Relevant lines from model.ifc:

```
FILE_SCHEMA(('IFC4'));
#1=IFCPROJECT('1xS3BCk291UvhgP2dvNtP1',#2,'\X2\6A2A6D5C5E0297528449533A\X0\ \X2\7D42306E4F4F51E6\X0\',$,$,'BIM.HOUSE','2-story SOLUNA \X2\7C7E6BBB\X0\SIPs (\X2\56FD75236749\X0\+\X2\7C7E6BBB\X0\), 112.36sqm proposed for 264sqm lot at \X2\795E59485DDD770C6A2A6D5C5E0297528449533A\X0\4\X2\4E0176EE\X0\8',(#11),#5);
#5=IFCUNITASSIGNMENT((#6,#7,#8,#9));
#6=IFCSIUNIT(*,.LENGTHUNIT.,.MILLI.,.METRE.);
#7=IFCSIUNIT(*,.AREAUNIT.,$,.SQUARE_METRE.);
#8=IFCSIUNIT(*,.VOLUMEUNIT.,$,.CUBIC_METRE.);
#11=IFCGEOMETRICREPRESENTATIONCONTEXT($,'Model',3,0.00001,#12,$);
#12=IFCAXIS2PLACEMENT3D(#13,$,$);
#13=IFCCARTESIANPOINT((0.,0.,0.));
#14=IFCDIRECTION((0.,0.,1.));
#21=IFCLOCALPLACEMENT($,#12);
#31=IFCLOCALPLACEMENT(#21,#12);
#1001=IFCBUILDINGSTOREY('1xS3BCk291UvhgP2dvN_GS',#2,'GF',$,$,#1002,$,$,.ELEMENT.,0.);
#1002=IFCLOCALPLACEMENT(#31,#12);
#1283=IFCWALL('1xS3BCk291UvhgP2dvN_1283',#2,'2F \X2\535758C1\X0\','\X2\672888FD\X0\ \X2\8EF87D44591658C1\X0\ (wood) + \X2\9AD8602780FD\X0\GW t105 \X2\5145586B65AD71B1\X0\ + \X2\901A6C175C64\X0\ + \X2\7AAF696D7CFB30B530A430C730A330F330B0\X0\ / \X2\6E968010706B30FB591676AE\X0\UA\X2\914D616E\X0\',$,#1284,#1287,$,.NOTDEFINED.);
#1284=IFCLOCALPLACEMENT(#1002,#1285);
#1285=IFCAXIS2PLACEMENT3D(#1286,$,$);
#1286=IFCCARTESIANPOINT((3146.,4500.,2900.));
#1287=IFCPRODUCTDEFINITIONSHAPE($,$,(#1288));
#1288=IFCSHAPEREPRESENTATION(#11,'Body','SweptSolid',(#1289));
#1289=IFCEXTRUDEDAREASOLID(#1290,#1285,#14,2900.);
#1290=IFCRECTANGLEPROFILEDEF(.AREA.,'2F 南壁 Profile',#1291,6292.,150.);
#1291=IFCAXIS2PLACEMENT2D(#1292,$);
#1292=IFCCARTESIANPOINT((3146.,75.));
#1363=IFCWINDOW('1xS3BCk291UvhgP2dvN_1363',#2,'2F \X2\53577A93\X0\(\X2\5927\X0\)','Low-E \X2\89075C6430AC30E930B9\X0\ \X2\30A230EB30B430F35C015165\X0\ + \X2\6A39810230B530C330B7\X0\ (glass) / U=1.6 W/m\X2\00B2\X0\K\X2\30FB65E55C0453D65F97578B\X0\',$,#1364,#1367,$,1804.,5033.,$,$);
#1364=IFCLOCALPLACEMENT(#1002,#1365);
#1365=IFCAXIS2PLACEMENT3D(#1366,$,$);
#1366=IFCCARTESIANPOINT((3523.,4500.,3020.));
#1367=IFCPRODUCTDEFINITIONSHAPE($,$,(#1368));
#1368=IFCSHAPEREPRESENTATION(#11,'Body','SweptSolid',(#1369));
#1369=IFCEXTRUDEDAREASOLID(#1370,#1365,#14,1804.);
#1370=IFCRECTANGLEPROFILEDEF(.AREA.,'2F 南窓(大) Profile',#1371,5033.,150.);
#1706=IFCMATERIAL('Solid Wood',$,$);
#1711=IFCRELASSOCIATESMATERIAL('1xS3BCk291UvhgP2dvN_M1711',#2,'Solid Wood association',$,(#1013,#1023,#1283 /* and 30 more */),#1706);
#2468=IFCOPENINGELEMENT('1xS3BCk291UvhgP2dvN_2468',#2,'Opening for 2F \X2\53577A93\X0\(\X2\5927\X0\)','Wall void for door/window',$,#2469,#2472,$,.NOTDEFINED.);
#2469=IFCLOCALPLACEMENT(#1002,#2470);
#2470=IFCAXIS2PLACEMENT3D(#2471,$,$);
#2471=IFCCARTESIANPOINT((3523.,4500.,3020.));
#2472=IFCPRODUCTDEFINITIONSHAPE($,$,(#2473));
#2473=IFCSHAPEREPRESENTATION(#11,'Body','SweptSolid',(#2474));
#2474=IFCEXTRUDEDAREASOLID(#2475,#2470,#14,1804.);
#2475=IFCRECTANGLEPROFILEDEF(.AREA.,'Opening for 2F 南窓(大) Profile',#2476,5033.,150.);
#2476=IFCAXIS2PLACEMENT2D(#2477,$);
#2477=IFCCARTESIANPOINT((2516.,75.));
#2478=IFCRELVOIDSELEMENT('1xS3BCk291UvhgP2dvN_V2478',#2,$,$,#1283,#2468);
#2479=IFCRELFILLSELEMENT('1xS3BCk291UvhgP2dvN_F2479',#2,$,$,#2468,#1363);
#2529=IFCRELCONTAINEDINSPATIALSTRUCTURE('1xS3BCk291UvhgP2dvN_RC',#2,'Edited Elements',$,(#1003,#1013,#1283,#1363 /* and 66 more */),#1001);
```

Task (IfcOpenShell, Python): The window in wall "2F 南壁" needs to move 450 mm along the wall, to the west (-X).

```python
import ifcopenshell
import ifcopenshell.api.geometry
import ifcopenshell.util.placement

model = ifcopenshell.open("model.ifc")

window = model.by_guid("1xS3BCk291UvhgP2dvN_1363")
opening = window.FillsVoids[0].RelatingOpeningElement
wall = opening.VoidsElements[0].RelatingBuildingElement

wall_matrix = ifcopenshell.util.placement.get_local_placement(wall.ObjectPlacement)
shift = wall_matrix[:3, 0] * -450.0
before = ifcopenshell.util.placement.get_local_placement(window.ObjectPlacement)[:3, 3].copy()

# The window is not placed relative to its opening, so move both.
for product in (opening, window):
    matrix = ifcopenshell.util.placement.get_local_placement(product.ObjectPlacement)
    matrix[:3, 3] += shift
    ifcopenshell.api.geometry.edit_object_placement(model, product=product, matrix=matrix, is_si=False)

after = ifcopenshell.util.placement.get_local_placement(window.ObjectPlacement)[:3, 3]
print("window moved by", (after - before).round(3) + 0.0)

model.write("model_updated.ifc")
```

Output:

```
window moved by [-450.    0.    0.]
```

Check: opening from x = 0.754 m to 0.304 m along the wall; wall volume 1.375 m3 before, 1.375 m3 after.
